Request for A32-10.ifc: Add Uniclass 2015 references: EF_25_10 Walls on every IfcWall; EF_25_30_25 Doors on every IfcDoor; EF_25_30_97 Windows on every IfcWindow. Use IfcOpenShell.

First a look at what the model holds.

```python
import ifcopenshell

model = ifcopenshell.open("A32-10.ifc")
print(model.schema)
print("classifications:", [c.Name for c in model.by_type("IfcClassification")])
for ifc_class in ("IfcDoor", "IfcRoof", "IfcStair", "IfcWall", "IfcWindow"):
    print(ifc_class, len(model.by_type(ifc_class)))
```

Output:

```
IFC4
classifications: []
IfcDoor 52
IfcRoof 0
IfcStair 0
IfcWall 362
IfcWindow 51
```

```python
import ifcopenshell
import ifcopenshell.api.classification

model = ifcopenshell.open("A32-10.ifc")

system = ifcopenshell.api.classification.add_classification(model, classification="Uniclass 2015")

codes = {
    "IfcWall": ("EF_25_10", "Walls"),
    "IfcDoor": ("EF_25_30_25", "Doors"),
    "IfcWindow": ("EF_25_30_97", "Windows"),
}
for ifc_class, (code, name) in codes.items():
    products = model.by_type(ifc_class)
    ifcopenshell.api.classification.add_reference(
        model, products=products, classification=system, identification=code, name=name
    )
    print(code, len(products))

model.write("A32-10-out.ifc")
```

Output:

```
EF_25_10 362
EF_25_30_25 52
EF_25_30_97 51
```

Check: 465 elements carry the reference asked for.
